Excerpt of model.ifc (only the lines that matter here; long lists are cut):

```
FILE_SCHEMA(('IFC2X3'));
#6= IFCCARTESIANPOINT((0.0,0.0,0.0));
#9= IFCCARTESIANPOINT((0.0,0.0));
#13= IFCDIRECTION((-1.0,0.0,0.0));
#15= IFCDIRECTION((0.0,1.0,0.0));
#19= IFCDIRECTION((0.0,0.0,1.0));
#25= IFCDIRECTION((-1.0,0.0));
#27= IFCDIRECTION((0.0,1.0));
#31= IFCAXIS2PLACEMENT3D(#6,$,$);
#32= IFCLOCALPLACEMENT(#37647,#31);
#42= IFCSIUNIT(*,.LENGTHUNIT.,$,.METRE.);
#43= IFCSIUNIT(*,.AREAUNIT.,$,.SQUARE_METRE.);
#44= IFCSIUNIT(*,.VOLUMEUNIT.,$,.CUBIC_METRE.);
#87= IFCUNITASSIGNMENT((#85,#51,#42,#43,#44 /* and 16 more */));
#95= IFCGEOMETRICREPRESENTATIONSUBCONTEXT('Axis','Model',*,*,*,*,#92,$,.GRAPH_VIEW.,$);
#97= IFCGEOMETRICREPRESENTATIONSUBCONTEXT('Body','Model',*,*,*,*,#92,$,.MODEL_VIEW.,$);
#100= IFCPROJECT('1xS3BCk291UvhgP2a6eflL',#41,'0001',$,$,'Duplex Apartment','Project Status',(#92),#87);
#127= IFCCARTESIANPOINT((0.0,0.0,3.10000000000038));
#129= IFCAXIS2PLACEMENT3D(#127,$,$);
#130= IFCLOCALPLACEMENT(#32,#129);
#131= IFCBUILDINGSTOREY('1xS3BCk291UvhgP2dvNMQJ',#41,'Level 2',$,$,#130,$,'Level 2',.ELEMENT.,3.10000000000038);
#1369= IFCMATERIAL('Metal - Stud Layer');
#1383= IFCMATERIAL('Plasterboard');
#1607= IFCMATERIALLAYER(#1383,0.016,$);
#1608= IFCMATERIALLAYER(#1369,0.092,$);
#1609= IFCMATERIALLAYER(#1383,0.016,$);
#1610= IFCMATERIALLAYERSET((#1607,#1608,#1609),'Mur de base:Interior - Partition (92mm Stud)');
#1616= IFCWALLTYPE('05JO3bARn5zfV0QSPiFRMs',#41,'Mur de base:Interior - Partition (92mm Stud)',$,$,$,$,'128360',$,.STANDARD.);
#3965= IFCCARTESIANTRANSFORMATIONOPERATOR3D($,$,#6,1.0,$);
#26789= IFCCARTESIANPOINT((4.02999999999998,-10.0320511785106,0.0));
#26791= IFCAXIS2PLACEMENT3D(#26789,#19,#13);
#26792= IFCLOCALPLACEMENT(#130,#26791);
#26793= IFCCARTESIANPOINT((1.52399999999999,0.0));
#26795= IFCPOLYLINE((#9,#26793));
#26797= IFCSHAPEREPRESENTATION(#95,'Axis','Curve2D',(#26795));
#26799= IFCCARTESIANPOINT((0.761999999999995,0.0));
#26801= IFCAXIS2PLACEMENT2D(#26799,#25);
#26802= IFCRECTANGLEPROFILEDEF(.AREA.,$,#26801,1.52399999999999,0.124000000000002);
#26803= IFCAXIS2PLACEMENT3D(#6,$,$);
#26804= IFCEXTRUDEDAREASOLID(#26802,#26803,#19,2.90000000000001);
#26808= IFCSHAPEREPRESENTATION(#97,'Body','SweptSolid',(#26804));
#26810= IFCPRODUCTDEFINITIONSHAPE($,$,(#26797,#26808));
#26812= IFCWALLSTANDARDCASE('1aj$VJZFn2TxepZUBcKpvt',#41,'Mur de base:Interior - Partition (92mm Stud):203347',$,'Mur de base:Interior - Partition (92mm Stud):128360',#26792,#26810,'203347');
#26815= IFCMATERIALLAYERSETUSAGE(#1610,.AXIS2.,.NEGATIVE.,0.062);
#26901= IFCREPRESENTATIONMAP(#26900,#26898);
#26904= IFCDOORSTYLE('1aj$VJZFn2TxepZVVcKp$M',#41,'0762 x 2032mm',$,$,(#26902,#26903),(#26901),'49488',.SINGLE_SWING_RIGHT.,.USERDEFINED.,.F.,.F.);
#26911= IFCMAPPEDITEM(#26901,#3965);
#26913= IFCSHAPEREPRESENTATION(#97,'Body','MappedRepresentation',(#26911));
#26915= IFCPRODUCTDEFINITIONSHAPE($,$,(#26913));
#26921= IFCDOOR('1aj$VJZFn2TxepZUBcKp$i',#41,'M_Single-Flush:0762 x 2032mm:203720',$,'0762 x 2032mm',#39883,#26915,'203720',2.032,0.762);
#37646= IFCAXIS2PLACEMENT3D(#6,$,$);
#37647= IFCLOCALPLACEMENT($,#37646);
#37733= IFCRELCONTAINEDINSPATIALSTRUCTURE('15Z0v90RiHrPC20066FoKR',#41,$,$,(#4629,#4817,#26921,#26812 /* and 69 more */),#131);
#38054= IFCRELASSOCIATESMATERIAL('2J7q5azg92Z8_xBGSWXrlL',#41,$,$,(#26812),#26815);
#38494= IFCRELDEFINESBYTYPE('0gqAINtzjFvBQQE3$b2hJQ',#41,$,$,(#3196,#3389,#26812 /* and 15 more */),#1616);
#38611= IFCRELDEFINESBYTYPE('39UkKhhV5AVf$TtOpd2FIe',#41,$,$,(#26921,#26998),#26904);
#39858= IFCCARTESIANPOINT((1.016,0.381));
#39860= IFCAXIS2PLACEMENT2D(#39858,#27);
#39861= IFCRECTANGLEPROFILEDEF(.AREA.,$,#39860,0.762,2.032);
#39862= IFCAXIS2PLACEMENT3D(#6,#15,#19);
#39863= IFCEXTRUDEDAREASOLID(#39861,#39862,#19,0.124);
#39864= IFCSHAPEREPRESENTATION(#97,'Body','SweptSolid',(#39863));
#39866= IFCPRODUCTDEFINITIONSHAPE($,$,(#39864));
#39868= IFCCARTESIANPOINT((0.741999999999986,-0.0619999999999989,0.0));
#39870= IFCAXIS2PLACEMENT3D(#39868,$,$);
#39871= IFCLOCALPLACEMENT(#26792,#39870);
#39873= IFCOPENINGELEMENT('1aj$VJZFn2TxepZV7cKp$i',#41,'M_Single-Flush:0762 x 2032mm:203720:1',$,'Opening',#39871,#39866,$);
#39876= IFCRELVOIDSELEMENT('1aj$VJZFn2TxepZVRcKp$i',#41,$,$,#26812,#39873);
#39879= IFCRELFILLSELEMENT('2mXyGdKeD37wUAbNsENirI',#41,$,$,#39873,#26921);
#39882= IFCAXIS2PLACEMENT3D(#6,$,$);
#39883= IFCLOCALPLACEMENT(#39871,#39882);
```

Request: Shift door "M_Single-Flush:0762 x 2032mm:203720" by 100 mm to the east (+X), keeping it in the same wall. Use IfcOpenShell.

```python
import ifcopenshell
import ifcopenshell.api.geometry
import ifcopenshell.util.placement
import ifcopenshell.util.unit

model = ifcopenshell.open("model.ifc")
unit_scale = ifcopenshell.util.unit.calculate_unit_scale(model)

door = model.by_id(26921)
opening = door.FillsVoids[0].RelatingOpeningElement
wall = opening.VoidsElements[0].RelatingBuildingElement

wall_matrix = ifcopenshell.util.placement.get_local_placement(wall.ObjectPlacement)
shift = wall_matrix[:3, 0] * -0.1 / unit_scale
before = ifcopenshell.util.placement.get_local_placement(door.ObjectPlacement)[:3, 3].copy()

# The door is placed relative to its opening, so it follows when the opening moves.
matrix = ifcopenshell.util.placement.get_local_placement(opening.ObjectPlacement)
matrix[:3, 3] += shift
ifcopenshell.api.geometry.edit_object_placement(
    model, product=opening, matrix=matrix, is_si=False, should_transform_children=True
)

after = ifcopenshell.util.placement.get_local_placement(door.ObjectPlacement)[:3, 3]
print("door moved by", (after - before).round(3) + 0.0)

model.write("model_rev.ifc")
```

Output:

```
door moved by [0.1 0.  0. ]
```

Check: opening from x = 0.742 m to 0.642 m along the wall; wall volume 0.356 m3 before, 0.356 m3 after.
